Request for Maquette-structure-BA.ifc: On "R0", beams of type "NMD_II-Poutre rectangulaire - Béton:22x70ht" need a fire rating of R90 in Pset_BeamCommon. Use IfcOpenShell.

First a look at what the model holds.

```python
import ifcopenshell
import ifcopenshell.util.element

model = ifcopenshell.open("Maquette-structure-BA.ifc")
print(model.schema)
storey = next(s for s in model.by_type("IfcBuildingStorey") if s.Name == "R0")
beams = [e for e in ifcopenshell.util.element.get_decomposition(storey) if e.is_a("IfcBeam")]
seen = {}
for e in beams:
    element_type = ifcopenshell.util.element.get_type(e)
    key = (element_type.Name if element_type != e and element_type else None, ifcopenshell.util.element.get_pset(e, "Pset_BeamCommon", "FireRating"))
    seen[key] = seen.get(key, 0) + 1
for (name, value), count in sorted(seen.items(), key=str):
    print(count, "x", name, "|", value)
```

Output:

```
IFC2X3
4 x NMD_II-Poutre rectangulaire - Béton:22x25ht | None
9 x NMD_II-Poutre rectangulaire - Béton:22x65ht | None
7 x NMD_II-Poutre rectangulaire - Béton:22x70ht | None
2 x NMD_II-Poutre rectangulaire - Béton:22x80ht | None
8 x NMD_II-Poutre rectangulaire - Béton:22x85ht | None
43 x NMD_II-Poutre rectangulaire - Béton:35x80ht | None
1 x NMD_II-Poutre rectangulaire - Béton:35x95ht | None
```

```python
import ifcopenshell
import ifcopenshell.api.pset
import ifcopenshell.util.element

model = ifcopenshell.open("Maquette-structure-BA.ifc")

storey = next(s for s in model.by_type("IfcBuildingStorey") if s.Name == "R0")
beams = [e for e in ifcopenshell.util.element.get_decomposition(storey) if e.is_a("IfcBeam")]

count = 0
for e in beams:
    element_type = ifcopenshell.util.element.get_type(e)
    if element_type in (None, e) or element_type.Name != "NMD_II-Poutre rectangulaire - Béton:22x70ht":
        continue
    # add_pset returns the element's existing set when there is one.
    pset = ifcopenshell.api.pset.add_pset(model, product=e, name="Pset_BeamCommon")
    ifcopenshell.api.pset.edit_pset(model, pset=pset, properties={"FireRating": "R90"})
    count += 1

print(count, "beams updated")

model.write("Maquette-structure-BA_rev.ifc")
```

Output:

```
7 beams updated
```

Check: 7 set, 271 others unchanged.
